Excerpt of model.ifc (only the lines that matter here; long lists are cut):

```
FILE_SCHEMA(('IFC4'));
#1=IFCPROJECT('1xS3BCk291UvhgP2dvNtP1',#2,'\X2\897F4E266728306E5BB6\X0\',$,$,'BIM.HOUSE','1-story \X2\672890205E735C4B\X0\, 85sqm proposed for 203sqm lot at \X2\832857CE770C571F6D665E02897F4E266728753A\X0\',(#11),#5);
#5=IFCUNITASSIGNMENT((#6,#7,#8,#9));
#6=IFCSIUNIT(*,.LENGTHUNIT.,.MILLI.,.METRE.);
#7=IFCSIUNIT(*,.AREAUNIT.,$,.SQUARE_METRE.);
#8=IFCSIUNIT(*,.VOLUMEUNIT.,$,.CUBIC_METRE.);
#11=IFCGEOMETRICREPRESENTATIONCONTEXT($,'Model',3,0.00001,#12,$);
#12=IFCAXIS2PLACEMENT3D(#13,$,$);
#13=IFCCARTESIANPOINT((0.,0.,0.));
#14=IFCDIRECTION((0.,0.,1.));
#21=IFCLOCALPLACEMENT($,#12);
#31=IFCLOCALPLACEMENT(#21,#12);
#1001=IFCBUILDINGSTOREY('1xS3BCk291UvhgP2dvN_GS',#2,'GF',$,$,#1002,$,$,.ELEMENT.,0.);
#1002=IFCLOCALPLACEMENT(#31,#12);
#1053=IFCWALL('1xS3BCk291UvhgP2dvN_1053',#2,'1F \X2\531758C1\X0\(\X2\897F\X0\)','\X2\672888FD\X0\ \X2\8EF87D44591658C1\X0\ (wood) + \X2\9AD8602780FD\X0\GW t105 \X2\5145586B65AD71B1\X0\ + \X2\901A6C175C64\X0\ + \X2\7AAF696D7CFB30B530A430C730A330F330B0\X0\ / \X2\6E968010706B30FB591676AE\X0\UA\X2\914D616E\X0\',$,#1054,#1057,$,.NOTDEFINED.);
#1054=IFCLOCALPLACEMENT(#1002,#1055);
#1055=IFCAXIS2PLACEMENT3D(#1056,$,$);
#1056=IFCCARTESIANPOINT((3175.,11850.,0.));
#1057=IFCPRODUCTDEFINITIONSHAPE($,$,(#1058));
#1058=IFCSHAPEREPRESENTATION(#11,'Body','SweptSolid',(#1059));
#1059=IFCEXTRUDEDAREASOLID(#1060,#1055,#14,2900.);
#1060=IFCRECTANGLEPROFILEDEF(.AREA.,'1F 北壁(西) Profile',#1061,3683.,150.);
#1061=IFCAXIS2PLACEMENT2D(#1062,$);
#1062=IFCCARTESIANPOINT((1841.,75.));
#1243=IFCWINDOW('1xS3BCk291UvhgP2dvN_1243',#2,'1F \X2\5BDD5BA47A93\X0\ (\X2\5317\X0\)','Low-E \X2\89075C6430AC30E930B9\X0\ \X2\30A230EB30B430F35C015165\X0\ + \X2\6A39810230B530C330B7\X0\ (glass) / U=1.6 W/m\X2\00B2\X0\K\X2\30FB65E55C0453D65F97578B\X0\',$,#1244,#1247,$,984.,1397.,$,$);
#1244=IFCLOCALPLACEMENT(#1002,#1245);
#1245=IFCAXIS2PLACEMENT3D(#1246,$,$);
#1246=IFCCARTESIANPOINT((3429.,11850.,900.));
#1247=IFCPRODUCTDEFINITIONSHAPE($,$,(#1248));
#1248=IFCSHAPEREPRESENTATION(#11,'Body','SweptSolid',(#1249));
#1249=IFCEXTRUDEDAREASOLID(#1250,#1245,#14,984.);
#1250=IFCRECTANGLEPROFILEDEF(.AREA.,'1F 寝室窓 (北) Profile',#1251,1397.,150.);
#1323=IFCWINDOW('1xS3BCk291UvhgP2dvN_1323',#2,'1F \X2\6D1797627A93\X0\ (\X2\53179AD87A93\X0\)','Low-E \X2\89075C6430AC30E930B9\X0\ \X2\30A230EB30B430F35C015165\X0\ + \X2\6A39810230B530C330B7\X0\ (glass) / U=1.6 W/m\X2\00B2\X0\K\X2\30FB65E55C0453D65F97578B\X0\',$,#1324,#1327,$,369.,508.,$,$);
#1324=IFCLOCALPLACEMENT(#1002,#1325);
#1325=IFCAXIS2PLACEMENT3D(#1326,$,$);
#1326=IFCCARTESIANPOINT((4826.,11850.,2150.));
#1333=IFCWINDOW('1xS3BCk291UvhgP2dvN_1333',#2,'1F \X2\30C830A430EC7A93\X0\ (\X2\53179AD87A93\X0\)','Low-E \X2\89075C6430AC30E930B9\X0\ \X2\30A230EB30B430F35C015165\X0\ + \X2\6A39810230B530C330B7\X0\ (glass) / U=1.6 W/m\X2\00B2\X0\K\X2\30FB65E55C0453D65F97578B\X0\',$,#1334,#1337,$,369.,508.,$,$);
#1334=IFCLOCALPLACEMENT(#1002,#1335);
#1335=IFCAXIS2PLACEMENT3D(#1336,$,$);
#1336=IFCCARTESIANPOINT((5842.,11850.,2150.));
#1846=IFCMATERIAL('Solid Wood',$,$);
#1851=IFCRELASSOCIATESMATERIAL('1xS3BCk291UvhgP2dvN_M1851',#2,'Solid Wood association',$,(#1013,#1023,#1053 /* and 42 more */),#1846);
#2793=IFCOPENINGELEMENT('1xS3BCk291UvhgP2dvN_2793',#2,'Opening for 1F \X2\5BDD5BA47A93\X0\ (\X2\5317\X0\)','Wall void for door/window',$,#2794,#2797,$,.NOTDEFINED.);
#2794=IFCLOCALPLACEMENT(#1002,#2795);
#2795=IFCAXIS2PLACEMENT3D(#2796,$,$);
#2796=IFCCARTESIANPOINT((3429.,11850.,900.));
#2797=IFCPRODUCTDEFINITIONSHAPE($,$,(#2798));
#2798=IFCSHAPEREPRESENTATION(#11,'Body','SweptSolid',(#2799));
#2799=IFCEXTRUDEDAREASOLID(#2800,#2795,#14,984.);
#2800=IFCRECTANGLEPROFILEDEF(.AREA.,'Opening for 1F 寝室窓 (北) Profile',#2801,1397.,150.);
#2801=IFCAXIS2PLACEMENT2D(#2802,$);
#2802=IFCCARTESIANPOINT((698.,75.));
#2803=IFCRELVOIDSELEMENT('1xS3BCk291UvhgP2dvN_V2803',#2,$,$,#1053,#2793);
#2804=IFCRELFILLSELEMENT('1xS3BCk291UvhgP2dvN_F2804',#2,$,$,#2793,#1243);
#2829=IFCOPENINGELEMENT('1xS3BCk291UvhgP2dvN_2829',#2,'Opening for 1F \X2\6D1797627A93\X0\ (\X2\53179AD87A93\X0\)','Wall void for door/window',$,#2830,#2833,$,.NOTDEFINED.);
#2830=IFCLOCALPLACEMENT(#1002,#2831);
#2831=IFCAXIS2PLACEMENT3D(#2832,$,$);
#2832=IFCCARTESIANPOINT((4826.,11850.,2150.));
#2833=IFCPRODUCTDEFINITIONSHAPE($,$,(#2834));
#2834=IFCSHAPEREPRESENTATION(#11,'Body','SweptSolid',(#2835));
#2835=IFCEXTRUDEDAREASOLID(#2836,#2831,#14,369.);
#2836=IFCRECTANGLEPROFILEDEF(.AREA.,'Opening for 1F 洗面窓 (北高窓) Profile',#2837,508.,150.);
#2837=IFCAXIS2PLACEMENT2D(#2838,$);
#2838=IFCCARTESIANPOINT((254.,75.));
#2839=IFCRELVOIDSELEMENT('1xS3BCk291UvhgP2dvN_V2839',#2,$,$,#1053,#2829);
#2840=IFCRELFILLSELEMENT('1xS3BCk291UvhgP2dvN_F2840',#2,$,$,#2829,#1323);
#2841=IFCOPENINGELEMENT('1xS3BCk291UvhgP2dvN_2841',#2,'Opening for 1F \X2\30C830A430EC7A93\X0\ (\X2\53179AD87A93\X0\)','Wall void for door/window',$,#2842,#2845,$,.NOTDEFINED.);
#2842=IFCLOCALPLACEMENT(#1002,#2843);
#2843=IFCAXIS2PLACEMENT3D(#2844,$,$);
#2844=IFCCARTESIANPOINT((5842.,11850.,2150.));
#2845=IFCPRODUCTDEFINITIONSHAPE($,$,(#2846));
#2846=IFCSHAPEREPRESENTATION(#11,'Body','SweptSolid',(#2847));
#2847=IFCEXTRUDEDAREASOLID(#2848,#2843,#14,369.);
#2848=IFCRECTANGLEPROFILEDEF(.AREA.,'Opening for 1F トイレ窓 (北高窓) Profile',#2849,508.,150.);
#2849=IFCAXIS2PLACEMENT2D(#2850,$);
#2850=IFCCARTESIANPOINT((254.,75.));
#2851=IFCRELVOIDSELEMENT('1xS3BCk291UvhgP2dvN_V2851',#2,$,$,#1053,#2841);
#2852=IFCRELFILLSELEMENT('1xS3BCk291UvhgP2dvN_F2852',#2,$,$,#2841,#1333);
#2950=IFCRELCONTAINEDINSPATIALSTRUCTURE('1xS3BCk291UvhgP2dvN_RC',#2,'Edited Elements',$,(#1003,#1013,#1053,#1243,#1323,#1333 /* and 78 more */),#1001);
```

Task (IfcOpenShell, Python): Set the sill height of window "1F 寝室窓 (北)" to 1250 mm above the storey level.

```python
import numpy as np
import ifcopenshell
import ifcopenshell.api.geometry
import ifcopenshell.geom
import ifcopenshell.util.element
import ifcopenshell.util.placement
import ifcopenshell.util.shape
import ifcopenshell.util.unit

model = ifcopenshell.open("model.ifc")
unit_scale = ifcopenshell.util.unit.calculate_unit_scale(model)

window = model.by_guid("1xS3BCk291UvhgP2dvN_1243")
opening = window.FillsVoids[0].RelatingOpeningElement
storey = ifcopenshell.util.element.get_container(window, ifc_class="IfcBuildingStorey")
level = ifcopenshell.util.placement.get_local_placement(storey.ObjectPlacement)[2, 3]

# The opening's origin need not be at the sill, so measure its lowest point.
shape = ifcopenshell.geom.create_shape(ifcopenshell.geom.settings(), opening)
bottom = ifcopenshell.util.shape.get_shape_bottom_elevation(shape, shape.geometry) / unit_scale
dz = level + 1.25 / unit_scale - bottom

shift = np.array([0.0, 0.0, dz])
# The window is not placed relative to its opening, so move both.
for product in (opening, window):
    matrix = ifcopenshell.util.placement.get_local_placement(product.ObjectPlacement)
    matrix[:3, 3] += shift
    ifcopenshell.api.geometry.edit_object_placement(model, product=product, matrix=matrix, is_si=False)

print(f"moved by {dz * unit_scale:+.3f} m")

model.write("model_v2.ifc")
```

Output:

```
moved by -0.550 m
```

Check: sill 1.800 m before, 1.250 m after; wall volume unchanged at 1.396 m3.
